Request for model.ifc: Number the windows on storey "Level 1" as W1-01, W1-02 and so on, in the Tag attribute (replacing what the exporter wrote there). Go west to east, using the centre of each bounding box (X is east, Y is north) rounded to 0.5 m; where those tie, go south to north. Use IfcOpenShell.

First a look at what the model holds.

```python
import ifcopenshell
import ifcopenshell.util.element
import ifcopenshell.util.placement

model = ifcopenshell.open("model.ifc")
print(model.schema)
storey = next(s for s in model.by_type("IfcBuildingStorey") if s.Name == "Level 1")
windows = [e for e in ifcopenshell.util.element.get_decomposition(storey) if e.is_a("IfcWindow")]
for e in sorted(windows, key=lambda e: e.id()):
    origin = ifcopenshell.util.placement.get_local_placement(e.ObjectPlacement)[:3, 3]
    print(e.id(), e.Tag, e.Name, origin.round(2) + 0.0, sep=" | ")
```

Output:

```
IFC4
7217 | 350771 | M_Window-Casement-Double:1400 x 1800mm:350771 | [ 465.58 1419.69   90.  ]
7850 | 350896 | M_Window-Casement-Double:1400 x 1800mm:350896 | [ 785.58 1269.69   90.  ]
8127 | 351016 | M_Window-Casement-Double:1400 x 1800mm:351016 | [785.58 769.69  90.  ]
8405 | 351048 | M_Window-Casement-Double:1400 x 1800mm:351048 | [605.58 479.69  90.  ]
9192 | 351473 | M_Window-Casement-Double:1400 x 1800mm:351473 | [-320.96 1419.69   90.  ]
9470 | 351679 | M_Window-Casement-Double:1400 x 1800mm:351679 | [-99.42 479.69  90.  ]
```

```python
import ifcopenshell
import ifcopenshell.geom
import ifcopenshell.util.element
import ifcopenshell.util.shape

model = ifcopenshell.open("model.ifc")
settings = ifcopenshell.geom.settings()
settings.set("use-world-coords", True)


def centre(element):
    shape = ifcopenshell.geom.create_shape(settings, element)
    return ifcopenshell.util.shape.get_bbox_centroid(shape.geometry)


storey = next(s for s in model.by_type("IfcBuildingStorey") if s.Name == "Level 1")
windows = [e for e in ifcopenshell.util.element.get_decomposition(storey) if e.is_a("IfcWindow")]

# Insertion points can sit at a corner or the storey origin, so sort by the geometry (in metres).
centres = {e: centre(e) for e in windows}
windows.sort(key=lambda e: (round(centres[e][0] / 0.5), centres[e][1]))

for i, e in enumerate(windows, start=1):
    number = f"W1-{i:02d}"
    e.Tag = number
    print(e.id(), number)

model.write("model_edited.ifc")
```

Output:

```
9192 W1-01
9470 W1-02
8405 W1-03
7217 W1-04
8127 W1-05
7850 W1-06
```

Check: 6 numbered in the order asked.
